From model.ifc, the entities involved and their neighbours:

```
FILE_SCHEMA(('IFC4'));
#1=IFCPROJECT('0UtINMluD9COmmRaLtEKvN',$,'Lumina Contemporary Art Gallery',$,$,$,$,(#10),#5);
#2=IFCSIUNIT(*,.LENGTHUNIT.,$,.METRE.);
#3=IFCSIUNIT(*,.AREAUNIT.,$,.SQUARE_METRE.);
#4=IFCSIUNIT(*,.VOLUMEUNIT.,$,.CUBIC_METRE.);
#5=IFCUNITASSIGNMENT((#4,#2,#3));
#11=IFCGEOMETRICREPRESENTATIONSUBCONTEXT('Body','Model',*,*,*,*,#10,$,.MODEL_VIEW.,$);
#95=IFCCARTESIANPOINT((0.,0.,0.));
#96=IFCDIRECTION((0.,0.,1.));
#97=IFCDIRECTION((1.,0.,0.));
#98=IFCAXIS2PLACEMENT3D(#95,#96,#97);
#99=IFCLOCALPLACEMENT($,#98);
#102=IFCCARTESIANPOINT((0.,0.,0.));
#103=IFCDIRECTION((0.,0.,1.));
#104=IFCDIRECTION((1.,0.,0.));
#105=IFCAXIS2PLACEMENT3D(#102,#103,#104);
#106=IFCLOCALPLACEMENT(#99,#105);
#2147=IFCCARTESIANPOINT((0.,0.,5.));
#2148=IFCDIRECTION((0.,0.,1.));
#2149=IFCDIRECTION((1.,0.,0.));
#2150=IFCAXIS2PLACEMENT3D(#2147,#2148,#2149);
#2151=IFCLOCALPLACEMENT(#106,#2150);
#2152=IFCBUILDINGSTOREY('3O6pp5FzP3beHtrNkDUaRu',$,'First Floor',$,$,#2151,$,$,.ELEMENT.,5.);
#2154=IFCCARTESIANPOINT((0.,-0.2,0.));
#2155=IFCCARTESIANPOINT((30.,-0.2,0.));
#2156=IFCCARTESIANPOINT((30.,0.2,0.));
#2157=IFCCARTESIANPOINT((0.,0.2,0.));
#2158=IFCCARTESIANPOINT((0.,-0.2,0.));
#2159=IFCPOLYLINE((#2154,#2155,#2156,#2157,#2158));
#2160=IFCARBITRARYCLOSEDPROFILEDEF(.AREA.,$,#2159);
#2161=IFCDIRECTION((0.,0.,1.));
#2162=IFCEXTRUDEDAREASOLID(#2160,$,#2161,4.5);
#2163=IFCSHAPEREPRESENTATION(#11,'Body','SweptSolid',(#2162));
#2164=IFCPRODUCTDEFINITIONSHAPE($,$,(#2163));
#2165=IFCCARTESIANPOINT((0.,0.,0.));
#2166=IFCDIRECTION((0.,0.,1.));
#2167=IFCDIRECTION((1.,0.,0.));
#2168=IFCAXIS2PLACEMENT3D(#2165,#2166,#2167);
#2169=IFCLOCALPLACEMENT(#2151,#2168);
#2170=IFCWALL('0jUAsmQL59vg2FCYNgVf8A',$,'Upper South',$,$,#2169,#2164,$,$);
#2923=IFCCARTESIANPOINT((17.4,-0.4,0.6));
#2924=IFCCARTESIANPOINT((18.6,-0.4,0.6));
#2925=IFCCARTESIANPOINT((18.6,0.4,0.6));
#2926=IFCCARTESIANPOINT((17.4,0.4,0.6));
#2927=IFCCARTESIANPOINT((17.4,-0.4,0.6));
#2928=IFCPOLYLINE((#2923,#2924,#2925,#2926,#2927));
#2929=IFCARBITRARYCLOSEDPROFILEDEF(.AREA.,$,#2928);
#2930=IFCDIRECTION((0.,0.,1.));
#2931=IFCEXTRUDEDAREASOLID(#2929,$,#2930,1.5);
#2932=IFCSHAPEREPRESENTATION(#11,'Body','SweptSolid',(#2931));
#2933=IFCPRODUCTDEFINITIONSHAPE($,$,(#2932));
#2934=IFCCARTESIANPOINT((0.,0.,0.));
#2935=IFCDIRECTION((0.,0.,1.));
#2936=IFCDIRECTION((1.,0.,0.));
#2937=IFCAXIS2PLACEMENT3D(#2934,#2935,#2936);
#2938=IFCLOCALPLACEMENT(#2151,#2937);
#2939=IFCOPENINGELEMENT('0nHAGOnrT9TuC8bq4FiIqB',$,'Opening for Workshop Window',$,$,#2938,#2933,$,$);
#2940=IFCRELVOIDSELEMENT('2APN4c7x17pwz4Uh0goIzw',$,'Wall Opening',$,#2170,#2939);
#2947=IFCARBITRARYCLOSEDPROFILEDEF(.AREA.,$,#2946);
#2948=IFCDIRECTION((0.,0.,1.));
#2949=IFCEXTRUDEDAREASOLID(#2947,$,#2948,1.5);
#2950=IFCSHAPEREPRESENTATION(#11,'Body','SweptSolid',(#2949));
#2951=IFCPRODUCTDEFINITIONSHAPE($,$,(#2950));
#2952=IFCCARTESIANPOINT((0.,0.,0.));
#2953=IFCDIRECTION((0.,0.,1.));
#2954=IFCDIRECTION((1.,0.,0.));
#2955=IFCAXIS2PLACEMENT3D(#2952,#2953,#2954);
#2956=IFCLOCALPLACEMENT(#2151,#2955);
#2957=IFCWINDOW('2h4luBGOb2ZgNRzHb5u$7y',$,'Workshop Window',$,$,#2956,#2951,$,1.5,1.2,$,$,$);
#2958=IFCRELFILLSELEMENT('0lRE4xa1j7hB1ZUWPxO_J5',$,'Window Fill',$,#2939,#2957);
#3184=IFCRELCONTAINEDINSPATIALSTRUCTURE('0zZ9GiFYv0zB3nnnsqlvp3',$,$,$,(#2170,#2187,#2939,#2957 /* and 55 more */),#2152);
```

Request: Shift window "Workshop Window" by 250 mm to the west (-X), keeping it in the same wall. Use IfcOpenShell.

```python
import ifcopenshell
import ifcopenshell.api.geometry
import ifcopenshell.util.placement

model = ifcopenshell.open("model.ifc")

window = model.by_guid("2h4luBGOb2ZgNRzHb5u$7y")
opening = window.FillsVoids[0].RelatingOpeningElement
wall = opening.VoidsElements[0].RelatingBuildingElement

wall_matrix = ifcopenshell.util.placement.get_local_placement(wall.ObjectPlacement)
shift = wall_matrix[:3, 0] * -0.25
before = ifcopenshell.util.placement.get_local_placement(window.ObjectPlacement)[:3, 3].copy()

# The window is not placed relative to its opening, so move both.
for product in (opening, window):
    matrix = ifcopenshell.util.placement.get_local_placement(product.ObjectPlacement)
    matrix[:3, 3] += shift
    ifcopenshell.api.geometry.edit_object_placement(model, product=product, matrix=matrix, is_si=False)

after = ifcopenshell.util.placement.get_local_placement(window.ObjectPlacement)[:3, 3]
print("window moved by", (after - before).round(3) + 0.0)

model.write("model_rev.ifc")
```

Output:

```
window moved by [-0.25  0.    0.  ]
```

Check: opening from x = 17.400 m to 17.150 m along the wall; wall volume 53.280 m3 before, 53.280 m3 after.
